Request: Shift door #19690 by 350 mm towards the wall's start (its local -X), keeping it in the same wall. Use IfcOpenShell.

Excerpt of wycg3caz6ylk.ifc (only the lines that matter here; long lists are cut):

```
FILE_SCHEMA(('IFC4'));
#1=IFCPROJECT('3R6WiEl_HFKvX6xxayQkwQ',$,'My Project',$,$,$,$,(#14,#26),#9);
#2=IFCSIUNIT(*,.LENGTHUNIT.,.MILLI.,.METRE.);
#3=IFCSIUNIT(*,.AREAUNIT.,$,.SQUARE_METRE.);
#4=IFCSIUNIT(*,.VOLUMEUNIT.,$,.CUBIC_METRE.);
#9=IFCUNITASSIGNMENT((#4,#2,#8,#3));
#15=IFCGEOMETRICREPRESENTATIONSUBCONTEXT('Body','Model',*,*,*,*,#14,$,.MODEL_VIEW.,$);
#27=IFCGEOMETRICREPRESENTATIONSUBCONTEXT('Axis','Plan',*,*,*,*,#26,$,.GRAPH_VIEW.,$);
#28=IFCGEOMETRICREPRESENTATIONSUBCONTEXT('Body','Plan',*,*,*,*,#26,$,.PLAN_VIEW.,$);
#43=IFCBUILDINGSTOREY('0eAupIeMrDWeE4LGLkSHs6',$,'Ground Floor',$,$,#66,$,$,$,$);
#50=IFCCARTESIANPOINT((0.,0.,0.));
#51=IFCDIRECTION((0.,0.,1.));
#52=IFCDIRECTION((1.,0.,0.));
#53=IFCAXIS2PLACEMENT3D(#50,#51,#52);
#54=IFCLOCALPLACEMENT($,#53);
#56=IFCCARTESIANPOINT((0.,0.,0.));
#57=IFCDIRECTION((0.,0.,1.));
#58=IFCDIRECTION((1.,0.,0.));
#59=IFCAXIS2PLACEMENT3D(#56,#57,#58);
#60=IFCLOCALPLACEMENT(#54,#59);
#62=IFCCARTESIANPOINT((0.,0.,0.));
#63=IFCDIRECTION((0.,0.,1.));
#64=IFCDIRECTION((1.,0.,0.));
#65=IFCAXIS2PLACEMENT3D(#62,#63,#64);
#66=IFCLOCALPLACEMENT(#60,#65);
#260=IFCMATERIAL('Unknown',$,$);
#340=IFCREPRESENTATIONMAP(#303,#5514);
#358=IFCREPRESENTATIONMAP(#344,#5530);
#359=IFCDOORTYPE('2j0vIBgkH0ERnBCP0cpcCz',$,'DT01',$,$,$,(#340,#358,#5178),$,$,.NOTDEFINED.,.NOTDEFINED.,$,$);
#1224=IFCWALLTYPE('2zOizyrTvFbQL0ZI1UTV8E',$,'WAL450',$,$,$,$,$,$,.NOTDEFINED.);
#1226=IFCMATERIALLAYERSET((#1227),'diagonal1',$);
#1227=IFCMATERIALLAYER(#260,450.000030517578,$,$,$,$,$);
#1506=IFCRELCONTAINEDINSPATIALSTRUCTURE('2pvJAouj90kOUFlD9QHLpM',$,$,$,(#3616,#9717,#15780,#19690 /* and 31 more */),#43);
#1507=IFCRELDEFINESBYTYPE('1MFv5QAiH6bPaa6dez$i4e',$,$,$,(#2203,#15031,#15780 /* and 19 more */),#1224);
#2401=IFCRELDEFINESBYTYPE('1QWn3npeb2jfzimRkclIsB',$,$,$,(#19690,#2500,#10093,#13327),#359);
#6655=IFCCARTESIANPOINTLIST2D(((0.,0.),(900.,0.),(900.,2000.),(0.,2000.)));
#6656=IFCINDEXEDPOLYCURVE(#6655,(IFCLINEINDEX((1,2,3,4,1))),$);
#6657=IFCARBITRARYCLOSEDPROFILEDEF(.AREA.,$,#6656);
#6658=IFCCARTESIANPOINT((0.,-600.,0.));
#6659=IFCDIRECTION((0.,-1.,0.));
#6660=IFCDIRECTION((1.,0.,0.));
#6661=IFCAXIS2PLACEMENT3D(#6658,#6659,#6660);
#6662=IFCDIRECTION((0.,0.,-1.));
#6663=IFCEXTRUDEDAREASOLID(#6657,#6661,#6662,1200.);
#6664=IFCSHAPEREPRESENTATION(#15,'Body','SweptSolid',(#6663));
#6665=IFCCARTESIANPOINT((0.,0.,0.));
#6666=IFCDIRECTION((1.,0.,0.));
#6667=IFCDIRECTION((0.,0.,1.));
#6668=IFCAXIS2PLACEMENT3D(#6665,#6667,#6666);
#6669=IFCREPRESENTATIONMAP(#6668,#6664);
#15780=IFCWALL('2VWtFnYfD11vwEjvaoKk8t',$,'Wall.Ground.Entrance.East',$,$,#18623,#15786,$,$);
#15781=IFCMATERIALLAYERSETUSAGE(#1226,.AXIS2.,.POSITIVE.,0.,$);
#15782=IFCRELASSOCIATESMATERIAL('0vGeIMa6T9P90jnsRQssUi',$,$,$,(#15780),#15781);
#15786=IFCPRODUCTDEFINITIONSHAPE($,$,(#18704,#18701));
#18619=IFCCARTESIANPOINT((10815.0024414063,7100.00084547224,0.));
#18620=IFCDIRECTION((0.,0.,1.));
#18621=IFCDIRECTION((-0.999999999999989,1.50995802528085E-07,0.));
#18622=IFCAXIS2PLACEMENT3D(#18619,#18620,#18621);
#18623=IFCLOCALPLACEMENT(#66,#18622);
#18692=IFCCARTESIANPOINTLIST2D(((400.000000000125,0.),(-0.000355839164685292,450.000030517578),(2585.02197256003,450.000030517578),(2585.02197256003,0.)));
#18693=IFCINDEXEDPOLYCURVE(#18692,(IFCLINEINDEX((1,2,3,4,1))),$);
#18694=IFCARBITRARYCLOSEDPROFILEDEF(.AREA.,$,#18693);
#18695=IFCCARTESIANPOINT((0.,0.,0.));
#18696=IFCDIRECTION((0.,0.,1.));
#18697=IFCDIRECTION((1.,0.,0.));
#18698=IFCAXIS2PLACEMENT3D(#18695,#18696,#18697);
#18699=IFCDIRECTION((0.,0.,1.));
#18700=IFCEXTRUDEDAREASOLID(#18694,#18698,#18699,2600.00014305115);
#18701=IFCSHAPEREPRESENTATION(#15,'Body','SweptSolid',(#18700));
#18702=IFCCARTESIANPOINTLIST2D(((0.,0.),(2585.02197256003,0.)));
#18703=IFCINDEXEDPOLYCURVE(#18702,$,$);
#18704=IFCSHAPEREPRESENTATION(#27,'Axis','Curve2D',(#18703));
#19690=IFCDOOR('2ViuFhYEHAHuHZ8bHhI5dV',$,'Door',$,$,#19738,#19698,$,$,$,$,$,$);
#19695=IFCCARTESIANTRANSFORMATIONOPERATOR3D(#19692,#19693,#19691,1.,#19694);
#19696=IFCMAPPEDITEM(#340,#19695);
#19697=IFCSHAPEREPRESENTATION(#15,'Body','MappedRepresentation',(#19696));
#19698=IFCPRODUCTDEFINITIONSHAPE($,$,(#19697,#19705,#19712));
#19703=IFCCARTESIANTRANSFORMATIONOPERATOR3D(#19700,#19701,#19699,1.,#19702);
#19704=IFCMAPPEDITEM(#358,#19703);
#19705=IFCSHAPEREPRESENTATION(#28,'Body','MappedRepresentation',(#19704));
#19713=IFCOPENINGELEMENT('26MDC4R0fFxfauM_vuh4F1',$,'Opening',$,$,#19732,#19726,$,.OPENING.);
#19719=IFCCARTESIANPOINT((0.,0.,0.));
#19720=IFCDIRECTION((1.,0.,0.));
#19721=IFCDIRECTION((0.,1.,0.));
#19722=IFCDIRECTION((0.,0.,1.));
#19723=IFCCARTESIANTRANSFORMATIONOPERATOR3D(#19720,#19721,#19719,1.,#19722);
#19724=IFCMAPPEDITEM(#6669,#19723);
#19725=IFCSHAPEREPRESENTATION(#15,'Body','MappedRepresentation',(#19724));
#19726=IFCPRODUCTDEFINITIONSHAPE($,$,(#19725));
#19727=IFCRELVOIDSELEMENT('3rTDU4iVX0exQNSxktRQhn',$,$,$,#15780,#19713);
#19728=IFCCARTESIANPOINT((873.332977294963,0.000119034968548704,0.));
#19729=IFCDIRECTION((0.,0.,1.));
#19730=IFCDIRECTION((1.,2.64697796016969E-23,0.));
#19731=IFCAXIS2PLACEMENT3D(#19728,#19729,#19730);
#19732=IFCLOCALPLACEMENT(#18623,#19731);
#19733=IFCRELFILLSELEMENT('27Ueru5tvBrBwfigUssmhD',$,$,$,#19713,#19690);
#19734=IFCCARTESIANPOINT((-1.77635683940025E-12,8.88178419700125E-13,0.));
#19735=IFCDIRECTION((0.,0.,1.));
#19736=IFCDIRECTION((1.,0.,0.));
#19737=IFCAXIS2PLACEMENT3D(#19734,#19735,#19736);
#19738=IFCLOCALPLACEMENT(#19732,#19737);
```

```python
import ifcopenshell
import ifcopenshell.api.geometry
import ifcopenshell.util.placement

model = ifcopenshell.open("wycg3caz6ylk.ifc")

door = model.by_guid("2ViuFhYEHAHuHZ8bHhI5dV")
opening = door.FillsVoids[0].RelatingOpeningElement
wall = opening.VoidsElements[0].RelatingBuildingElement

wall_matrix = ifcopenshell.util.placement.get_local_placement(wall.ObjectPlacement)
shift = wall_matrix[:3, 0] * -350.0
before = ifcopenshell.util.placement.get_local_placement(door.ObjectPlacement)[:3, 3].copy()

# The door is placed relative to its opening, so it follows when the opening moves.
matrix = ifcopenshell.util.placement.get_local_placement(opening.ObjectPlacement)
matrix[:3, 3] += shift
ifcopenshell.api.geometry.edit_object_placement(
    model, product=opening, matrix=matrix, is_si=False, should_transform_children=True
)

after = ifcopenshell.util.placement.get_local_placement(door.ObjectPlacement)[:3, 3]
print("door moved by", (after - before).round(3) + 0.0)

model.write("wycg3caz6ylk_edited.ifc")
```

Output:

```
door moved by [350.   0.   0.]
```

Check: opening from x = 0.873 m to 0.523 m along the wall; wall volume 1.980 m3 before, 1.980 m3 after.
